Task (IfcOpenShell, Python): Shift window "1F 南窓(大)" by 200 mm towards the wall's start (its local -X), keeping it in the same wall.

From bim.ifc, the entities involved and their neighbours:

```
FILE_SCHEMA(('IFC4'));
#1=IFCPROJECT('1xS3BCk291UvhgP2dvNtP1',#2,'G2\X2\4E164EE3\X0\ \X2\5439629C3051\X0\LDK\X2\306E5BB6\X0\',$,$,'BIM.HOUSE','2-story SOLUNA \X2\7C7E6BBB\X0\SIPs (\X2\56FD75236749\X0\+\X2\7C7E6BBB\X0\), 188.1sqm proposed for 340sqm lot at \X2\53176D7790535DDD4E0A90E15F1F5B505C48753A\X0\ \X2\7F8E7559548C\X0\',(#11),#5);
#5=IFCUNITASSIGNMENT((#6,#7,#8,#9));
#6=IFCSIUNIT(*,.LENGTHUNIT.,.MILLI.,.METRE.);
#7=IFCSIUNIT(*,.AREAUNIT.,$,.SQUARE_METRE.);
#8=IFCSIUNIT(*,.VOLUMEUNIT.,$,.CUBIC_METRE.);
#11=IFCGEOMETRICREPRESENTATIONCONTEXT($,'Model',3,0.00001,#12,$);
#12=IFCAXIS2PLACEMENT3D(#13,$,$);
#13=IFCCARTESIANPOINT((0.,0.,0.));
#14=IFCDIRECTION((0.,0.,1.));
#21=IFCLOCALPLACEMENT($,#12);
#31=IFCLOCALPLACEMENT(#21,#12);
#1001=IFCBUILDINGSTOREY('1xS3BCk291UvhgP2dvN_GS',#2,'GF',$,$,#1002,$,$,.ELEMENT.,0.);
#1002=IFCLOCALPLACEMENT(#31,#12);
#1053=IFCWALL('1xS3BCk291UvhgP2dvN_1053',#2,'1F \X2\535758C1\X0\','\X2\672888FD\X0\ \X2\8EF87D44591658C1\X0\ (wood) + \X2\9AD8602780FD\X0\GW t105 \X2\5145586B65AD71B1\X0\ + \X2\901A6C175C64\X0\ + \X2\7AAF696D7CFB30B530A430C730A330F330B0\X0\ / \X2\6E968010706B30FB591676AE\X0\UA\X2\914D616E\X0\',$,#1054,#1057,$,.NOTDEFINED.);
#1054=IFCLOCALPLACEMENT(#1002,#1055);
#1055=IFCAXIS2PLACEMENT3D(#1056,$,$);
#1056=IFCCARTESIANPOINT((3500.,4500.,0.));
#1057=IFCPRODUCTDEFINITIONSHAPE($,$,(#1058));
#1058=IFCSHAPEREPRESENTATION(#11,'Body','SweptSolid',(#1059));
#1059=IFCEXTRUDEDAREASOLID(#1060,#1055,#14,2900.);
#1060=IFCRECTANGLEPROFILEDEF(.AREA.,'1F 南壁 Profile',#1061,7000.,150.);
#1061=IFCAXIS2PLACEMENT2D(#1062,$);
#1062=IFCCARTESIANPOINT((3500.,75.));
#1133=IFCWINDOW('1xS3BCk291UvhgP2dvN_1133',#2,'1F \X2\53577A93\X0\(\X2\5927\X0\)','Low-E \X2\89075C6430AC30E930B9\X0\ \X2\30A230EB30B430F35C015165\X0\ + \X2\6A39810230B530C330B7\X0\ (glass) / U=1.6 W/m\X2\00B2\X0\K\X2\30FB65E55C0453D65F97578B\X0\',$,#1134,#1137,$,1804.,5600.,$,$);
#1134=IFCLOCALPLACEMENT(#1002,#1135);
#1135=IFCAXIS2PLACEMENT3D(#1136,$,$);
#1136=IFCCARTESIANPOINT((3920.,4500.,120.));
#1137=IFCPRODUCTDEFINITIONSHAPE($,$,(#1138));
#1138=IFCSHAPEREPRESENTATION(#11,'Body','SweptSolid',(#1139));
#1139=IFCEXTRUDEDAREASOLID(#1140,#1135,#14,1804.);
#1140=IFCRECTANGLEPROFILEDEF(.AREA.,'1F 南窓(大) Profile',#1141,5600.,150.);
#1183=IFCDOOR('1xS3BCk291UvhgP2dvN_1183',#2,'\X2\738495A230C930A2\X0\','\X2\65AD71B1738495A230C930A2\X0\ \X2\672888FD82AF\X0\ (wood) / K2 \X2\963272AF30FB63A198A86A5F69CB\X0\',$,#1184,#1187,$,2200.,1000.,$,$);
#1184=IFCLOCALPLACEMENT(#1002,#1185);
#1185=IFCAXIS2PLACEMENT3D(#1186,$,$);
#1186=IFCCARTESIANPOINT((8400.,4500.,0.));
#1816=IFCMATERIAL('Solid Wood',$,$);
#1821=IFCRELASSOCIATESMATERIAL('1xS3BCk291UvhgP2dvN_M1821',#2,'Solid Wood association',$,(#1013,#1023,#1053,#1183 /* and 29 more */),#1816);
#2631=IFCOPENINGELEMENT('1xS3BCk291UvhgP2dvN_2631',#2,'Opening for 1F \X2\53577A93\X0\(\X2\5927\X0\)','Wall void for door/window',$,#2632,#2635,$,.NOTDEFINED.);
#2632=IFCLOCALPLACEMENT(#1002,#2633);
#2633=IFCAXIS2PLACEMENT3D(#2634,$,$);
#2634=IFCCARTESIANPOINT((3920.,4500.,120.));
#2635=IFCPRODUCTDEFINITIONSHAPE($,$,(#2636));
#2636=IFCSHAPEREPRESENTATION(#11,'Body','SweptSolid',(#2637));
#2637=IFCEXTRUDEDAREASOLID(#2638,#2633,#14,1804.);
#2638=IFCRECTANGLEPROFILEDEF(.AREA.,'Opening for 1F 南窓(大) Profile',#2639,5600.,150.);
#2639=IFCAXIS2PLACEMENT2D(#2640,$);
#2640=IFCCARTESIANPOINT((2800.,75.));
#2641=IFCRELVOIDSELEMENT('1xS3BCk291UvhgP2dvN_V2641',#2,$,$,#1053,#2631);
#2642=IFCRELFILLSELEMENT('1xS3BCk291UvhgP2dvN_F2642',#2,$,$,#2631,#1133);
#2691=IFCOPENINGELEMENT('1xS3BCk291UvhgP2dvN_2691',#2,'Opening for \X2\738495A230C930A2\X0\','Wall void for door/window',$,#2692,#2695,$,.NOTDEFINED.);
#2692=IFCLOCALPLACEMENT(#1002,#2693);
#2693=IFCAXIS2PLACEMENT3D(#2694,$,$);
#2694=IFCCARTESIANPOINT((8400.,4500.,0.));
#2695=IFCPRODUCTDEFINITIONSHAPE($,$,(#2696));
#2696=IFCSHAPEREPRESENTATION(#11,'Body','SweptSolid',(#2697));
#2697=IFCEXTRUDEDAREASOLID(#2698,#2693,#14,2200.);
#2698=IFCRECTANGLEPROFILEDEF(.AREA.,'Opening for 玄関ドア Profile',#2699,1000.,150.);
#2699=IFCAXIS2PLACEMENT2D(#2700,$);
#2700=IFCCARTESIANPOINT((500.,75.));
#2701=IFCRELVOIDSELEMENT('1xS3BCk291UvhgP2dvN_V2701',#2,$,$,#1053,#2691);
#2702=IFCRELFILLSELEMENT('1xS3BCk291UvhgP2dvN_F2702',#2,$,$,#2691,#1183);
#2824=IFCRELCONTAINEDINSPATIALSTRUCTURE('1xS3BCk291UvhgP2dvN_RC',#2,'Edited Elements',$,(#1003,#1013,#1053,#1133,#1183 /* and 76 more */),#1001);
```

```python
import ifcopenshell
import ifcopenshell.api.geometry
import ifcopenshell.util.placement
import ifcopenshell.util.unit

model = ifcopenshell.open("bim.ifc")
unit_scale = ifcopenshell.util.unit.calculate_unit_scale(model)

window = model.by_guid("1xS3BCk291UvhgP2dvN_1133")
opening = window.FillsVoids[0].RelatingOpeningElement
wall = opening.VoidsElements[0].RelatingBuildingElement

wall_matrix = ifcopenshell.util.placement.get_local_placement(wall.ObjectPlacement)
shift = wall_matrix[:3, 0] * -0.2 / unit_scale
before = ifcopenshell.util.placement.get_local_placement(window.ObjectPlacement)[:3, 3].copy()

# The window is not placed relative to its opening, so move both.
for product in (opening, window):
    matrix = ifcopenshell.util.placement.get_local_placement(product.ObjectPlacement)
    matrix[:3, 3] += shift
    ifcopenshell.api.geometry.edit_object_placement(model, product=product, matrix=matrix, is_si=False)

after = ifcopenshell.util.placement.get_local_placement(window.ObjectPlacement)[:3, 3]
print("window moved by", (after - before).round(3) + 0.0)

model.write("bim_updated.ifc")
```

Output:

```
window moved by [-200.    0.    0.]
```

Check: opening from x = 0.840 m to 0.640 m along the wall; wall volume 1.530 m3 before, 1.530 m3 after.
